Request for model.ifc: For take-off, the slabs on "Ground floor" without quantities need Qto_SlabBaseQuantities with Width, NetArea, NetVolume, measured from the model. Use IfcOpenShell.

First a look at what the model holds.

```python
import ifcopenshell
import ifcopenshell.util.element
import ifcopenshell.util.unit

model = ifcopenshell.open("model.ifc")
print(model.schema)
for unit_type in ("LENGTHUNIT", "AREAUNIT", "VOLUMEUNIT"):
    print(unit_type, ifcopenshell.util.unit.calculate_unit_scale(model, unit_type))
storey = next(s for s in model.by_type("IfcBuildingStorey") if s.Name == "Ground floor")
slabs = [e for e in ifcopenshell.util.element.get_decomposition(storey) if e.is_a("IfcSlab")]
for e in sorted(slabs, key=lambda e: e.id()):
    print(e.id(), e.is_a(), e.Name, list(ifcopenshell.util.element.get_psets(e, qtos_only=True)), sep=" | ")
```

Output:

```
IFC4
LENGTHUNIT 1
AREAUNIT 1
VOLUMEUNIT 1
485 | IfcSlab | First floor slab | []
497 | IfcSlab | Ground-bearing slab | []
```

```python
import ifcopenshell
import ifcopenshell.api.pset
import ifcopenshell.geom
import ifcopenshell.util.element
import ifcopenshell.util.shape
import ifcopenshell.util.unit

model = ifcopenshell.open("model.ifc")
unit_scale = ifcopenshell.util.unit.calculate_unit_scale(model)
area_scale = ifcopenshell.util.unit.calculate_unit_scale(model, "AREAUNIT")
volume_scale = ifcopenshell.util.unit.calculate_unit_scale(model, "VOLUMEUNIT")
settings = ifcopenshell.geom.settings()

storey = next(s for s in model.by_type("IfcBuildingStorey") if s.Name == "Ground floor")
slabs = [e for e in ifcopenshell.util.element.get_decomposition(storey) if e.is_a("IfcSlab")]

for e in sorted(slabs, key=lambda e: e.id()):
    if ifcopenshell.util.element.get_psets(e, qtos_only=True, should_inherit=False):
        continue
    # Geometry comes back in metres, in the element's own axes.
    shape = ifcopenshell.geom.create_shape(settings, e)
    values = {
        "Width": ifcopenshell.util.shape.get_z(shape.geometry) / unit_scale,
        "NetArea": ifcopenshell.util.shape.get_footprint_area(shape.geometry) / area_scale,
        "NetVolume": ifcopenshell.util.shape.get_volume(shape.geometry) / volume_scale,
    }
    qto = ifcopenshell.api.pset.add_qto(model, product=e, name="Qto_SlabBaseQuantities")
    ifcopenshell.api.pset.edit_qto(model, qto=qto, properties=values)
    print(e.id(), {k: round(v, 3) for k, v in values.items()})

model.write("model-out.ifc")
```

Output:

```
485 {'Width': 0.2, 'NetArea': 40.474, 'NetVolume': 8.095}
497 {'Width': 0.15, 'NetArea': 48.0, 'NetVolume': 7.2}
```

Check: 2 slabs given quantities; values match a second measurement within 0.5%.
